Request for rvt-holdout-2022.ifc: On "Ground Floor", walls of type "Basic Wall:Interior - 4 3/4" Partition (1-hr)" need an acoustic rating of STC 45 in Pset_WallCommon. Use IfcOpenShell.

First a look at what the model holds.

```python
import ifcopenshell
import ifcopenshell.util.element

model = ifcopenshell.open("rvt-holdout-2022.ifc")
print(model.schema)
storey = next(s for s in model.by_type("IfcBuildingStorey") if s.Name == "Ground Floor")
walls = [e for e in ifcopenshell.util.element.get_decomposition(storey) if e.is_a("IfcWall")]
seen = {}
for e in walls:
    element_type = ifcopenshell.util.element.get_type(e)
    key = (element_type.Name if element_type != e and element_type else None, ifcopenshell.util.element.get_pset(e, "Pset_WallCommon", "AcousticRating"))
    seen[key] = seen.get(key, 0) + 1
for (name, value), count in sorted(seen.items(), key=str):
    print(count, "x", name, "|", value)
```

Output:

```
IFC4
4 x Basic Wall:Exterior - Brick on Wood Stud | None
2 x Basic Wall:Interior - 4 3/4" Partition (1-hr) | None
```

```python
import ifcopenshell
import ifcopenshell.api.pset
import ifcopenshell.util.element

model = ifcopenshell.open("rvt-holdout-2022.ifc")

storey = next(s for s in model.by_type("IfcBuildingStorey") if s.Name == "Ground Floor")
walls = [e for e in ifcopenshell.util.element.get_decomposition(storey) if e.is_a("IfcWall")]

count = 0
for e in walls:
    element_type = ifcopenshell.util.element.get_type(e)
    if element_type in (None, e) or element_type.Name != 'Basic Wall:Interior - 4 3/4" Partition (1-hr)':
        continue
    # add_pset returns the element's existing set when there is one.
    pset = ifcopenshell.api.pset.add_pset(model, product=e, name="Pset_WallCommon")
    ifcopenshell.api.pset.edit_pset(model, pset=pset, properties={"AcousticRating": "STC 45"})
    count += 1

print(count, "walls updated")

model.write("rvt-holdout-2022-out.ifc")
```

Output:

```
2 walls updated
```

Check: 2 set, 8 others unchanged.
